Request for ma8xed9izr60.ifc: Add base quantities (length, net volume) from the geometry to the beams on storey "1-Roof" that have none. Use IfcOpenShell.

First a look at what the model holds.

```python
import ifcopenshell
import ifcopenshell.util.element
import ifcopenshell.util.unit

model = ifcopenshell.open("ma8xed9izr60.ifc")
print(model.schema)
for unit_type in ("LENGTHUNIT", "AREAUNIT", "VOLUMEUNIT"):
    print(unit_type, ifcopenshell.util.unit.calculate_unit_scale(model, unit_type))
storey = next(s for s in model.by_type("IfcBuildingStorey") if s.Name == "1-Roof")
beams = [e for e in ifcopenshell.util.element.get_decomposition(storey) if e.is_a("IfcBeam")]
for e in sorted(beams, key=lambda e: e.id()):
    print(e.id(), e.is_a(), e.Name, list(ifcopenshell.util.element.get_psets(e, qtos_only=True)), sep=" | ")
```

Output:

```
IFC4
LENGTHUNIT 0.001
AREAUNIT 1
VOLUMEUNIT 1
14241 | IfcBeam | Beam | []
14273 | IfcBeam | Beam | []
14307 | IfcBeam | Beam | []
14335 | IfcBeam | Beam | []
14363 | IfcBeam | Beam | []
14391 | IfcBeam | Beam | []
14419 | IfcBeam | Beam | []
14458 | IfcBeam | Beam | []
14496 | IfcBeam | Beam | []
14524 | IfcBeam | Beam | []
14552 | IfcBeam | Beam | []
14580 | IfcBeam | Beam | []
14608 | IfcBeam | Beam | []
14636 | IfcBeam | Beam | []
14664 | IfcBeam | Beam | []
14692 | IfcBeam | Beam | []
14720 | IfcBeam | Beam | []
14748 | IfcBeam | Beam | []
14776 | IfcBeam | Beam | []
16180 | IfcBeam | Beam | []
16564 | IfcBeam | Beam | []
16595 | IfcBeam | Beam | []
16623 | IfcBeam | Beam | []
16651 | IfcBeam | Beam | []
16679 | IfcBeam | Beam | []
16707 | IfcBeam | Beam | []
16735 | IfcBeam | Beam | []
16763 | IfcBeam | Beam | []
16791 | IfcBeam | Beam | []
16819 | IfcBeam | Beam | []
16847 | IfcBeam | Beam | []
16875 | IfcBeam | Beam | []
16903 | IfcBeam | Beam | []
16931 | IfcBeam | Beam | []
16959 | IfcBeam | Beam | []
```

```python
import ifcopenshell
import ifcopenshell.api.pset
import ifcopenshell.geom
import ifcopenshell.util.element
import ifcopenshell.util.shape
import ifcopenshell.util.unit

model = ifcopenshell.open("ma8xed9izr60.ifc")
unit_scale = ifcopenshell.util.unit.calculate_unit_scale(model)
volume_scale = ifcopenshell.util.unit.calculate_unit_scale(model, "VOLUMEUNIT")
settings = ifcopenshell.geom.settings()

storey = next(s for s in model.by_type("IfcBuildingStorey") if s.Name == "1-Roof")
beams = [e for e in ifcopenshell.util.element.get_decomposition(storey) if e.is_a("IfcBeam")]

for e in sorted(beams, key=lambda e: e.id()):
    if ifcopenshell.util.element.get_psets(e, qtos_only=True, should_inherit=False):
        continue
    # Geometry comes back in metres, in the element's own axes.
    shape = ifcopenshell.geom.create_shape(settings, e)
    values = {
        "Length": ifcopenshell.util.shape.get_max_xyz(shape.geometry) / unit_scale,
        "NetVolume": ifcopenshell.util.shape.get_volume(shape.geometry) / volume_scale,
    }
    qto = ifcopenshell.api.pset.add_qto(model, product=e, name="Qto_BeamBaseQuantities")
    ifcopenshell.api.pset.edit_qto(model, qto=qto, properties=values)
    print(e.id(), {k: round(v, 3) for k, v in values.items()})

model.write("ma8xed9izr60_updated.ifc")
```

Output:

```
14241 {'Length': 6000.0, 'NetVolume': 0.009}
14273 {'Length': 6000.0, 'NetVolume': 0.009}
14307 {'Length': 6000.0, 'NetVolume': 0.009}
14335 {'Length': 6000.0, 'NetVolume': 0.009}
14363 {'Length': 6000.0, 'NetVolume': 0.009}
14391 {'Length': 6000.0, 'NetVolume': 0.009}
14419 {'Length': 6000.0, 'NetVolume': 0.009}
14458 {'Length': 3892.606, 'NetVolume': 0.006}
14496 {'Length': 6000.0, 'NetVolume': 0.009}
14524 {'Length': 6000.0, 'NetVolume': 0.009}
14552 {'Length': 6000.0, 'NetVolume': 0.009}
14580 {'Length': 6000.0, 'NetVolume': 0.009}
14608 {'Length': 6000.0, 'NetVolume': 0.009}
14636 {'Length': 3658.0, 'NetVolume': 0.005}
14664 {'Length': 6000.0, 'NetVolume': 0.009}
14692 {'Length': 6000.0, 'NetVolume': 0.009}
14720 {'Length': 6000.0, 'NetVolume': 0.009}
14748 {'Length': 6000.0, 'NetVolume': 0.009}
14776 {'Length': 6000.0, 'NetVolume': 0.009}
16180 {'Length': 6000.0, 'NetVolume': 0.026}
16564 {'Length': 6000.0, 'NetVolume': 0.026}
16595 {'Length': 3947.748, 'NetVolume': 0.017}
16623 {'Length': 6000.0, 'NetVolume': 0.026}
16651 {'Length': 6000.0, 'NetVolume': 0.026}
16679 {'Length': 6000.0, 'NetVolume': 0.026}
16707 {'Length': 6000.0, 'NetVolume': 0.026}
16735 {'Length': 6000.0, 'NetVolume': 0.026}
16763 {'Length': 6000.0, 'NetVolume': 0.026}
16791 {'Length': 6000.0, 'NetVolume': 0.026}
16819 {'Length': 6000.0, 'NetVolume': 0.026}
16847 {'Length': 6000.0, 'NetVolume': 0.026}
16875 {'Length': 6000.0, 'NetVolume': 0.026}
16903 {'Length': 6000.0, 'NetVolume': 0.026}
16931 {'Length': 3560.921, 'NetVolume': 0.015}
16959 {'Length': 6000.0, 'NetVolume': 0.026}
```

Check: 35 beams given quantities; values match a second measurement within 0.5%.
